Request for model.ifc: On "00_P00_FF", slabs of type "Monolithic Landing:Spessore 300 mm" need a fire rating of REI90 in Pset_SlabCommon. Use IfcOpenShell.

First a look at what the model holds.

```python
import ifcopenshell
import ifcopenshell.util.element

model = ifcopenshell.open("model.ifc")
print(model.schema)
storey = next(s for s in model.by_type("IfcBuildingStorey") if s.Name == "00_P00_FF")
slabs = [e for e in ifcopenshell.util.element.get_decomposition(storey) if e.is_a("IfcSlab")]
seen = {}
for e in slabs:
    element_type = ifcopenshell.util.element.get_type(e)
    key = (element_type.Name if element_type != e and element_type else None, ifcopenshell.util.element.get_pset(e, "Pset_SlabCommon", "FireRating"))
    seen[key] = seen.get(key, 0) + 1
for (name, value), count in sorted(seen.items(), key=str):
    print(count, "x", name, "|", value)
```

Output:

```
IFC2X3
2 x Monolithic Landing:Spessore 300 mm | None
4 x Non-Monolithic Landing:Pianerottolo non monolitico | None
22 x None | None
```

```python
import ifcopenshell
import ifcopenshell.api.pset
import ifcopenshell.util.element

model = ifcopenshell.open("model.ifc")

storey = next(s for s in model.by_type("IfcBuildingStorey") if s.Name == "00_P00_FF")
slabs = [e for e in ifcopenshell.util.element.get_decomposition(storey) if e.is_a("IfcSlab")]

count = 0
for e in slabs:
    element_type = ifcopenshell.util.element.get_type(e)
    if element_type in (None, e) or element_type.Name != "Monolithic Landing:Spessore 300 mm":
        continue
    # add_pset returns the element's existing set when there is one.
    pset = ifcopenshell.api.pset.add_pset(model, product=e, name="Pset_SlabCommon")
    ifcopenshell.api.pset.edit_pset(model, pset=pset, properties={"FireRating": "REI90"})
    count += 1

print(count, "slabs updated")

model.write("model_v2.ifc")
```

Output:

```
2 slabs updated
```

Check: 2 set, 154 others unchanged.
